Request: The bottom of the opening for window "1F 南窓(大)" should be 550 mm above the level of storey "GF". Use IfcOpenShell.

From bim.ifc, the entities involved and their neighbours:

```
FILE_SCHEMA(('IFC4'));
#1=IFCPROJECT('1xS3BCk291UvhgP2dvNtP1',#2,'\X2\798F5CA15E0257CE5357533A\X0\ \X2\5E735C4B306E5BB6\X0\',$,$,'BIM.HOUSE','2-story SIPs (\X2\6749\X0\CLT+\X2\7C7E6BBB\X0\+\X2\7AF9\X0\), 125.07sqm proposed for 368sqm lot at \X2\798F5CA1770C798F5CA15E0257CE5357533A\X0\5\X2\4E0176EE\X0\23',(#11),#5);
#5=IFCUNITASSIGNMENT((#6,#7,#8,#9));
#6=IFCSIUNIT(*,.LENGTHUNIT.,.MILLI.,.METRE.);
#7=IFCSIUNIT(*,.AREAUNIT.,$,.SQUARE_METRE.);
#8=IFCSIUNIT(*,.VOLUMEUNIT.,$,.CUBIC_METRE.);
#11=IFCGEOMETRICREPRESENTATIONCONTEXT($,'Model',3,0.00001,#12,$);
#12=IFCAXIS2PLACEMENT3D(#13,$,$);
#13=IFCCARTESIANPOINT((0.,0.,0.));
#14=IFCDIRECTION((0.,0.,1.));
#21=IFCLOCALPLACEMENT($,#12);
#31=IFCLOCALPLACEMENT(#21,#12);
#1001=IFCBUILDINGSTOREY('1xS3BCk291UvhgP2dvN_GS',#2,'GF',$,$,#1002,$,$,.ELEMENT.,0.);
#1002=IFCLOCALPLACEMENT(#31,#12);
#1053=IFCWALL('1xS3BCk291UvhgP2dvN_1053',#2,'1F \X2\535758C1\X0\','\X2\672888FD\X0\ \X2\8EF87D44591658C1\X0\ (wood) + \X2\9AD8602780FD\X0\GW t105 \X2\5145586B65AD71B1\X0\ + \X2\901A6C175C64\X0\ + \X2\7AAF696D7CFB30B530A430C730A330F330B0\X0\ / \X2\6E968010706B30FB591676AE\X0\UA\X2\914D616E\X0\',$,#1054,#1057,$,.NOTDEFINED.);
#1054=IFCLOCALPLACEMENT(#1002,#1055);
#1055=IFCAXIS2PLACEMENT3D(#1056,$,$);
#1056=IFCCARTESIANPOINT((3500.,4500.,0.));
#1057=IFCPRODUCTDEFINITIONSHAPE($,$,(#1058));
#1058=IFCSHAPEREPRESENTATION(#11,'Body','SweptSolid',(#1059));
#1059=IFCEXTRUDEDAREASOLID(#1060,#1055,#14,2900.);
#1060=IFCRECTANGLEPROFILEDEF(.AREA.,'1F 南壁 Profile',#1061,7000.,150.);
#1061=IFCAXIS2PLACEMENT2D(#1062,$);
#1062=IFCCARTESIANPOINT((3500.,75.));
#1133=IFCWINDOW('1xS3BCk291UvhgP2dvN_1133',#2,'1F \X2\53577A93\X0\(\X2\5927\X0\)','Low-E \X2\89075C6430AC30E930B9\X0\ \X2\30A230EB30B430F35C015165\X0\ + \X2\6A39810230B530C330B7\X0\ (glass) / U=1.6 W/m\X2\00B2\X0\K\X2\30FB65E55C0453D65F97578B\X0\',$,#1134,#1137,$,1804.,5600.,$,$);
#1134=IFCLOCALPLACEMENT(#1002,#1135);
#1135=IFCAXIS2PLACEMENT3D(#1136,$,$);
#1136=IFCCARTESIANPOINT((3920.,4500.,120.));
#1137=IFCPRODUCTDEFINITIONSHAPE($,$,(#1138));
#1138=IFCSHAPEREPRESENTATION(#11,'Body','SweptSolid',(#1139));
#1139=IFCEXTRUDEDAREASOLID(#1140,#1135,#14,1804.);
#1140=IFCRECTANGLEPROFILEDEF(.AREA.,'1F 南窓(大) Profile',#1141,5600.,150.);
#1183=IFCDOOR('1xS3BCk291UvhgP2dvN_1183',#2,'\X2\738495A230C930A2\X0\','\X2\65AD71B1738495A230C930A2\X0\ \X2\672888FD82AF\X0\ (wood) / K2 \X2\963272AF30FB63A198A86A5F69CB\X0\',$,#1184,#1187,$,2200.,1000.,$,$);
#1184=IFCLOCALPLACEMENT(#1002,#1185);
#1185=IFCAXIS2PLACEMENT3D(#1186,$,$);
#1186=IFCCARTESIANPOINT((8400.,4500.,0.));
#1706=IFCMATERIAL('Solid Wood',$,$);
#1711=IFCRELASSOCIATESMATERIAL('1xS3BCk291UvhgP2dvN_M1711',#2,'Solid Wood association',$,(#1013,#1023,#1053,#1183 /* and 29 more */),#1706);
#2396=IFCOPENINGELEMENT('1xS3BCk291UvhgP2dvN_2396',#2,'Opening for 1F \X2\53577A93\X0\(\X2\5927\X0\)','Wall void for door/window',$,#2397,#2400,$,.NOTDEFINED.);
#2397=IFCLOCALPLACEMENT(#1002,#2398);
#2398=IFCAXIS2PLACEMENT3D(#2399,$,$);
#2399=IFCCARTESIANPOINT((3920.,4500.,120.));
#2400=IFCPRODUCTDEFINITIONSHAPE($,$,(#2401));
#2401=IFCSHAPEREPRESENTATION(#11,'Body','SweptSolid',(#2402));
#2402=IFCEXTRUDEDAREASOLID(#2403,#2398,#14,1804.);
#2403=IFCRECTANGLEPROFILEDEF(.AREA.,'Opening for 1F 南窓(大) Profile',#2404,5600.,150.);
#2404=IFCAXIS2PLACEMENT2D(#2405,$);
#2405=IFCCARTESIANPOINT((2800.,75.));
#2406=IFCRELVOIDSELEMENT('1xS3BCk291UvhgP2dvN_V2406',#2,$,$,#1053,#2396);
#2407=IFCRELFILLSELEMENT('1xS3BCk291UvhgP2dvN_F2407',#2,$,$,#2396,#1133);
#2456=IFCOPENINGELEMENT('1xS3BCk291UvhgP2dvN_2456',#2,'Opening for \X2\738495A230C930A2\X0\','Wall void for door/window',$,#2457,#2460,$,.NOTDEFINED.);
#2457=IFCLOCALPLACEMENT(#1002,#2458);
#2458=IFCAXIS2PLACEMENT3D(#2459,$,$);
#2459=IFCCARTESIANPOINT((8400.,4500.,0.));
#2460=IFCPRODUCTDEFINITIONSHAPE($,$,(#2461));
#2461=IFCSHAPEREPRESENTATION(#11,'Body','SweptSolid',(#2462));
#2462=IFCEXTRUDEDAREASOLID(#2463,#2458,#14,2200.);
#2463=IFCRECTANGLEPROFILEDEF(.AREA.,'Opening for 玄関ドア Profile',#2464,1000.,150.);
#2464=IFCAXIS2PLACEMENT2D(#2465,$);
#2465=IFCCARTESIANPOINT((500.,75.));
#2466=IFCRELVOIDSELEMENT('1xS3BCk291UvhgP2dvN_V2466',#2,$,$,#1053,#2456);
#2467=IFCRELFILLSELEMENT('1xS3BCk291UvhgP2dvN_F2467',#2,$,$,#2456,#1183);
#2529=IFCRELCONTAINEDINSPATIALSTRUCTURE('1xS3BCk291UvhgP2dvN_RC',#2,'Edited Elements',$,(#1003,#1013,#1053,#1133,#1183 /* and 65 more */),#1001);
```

```python
import numpy as np
import ifcopenshell
import ifcopenshell.api.geometry
import ifcopenshell.geom
import ifcopenshell.util.element
import ifcopenshell.util.placement
import ifcopenshell.util.shape
import ifcopenshell.util.unit

model = ifcopenshell.open("bim.ifc")
unit_scale = ifcopenshell.util.unit.calculate_unit_scale(model)

window = model.by_guid("1xS3BCk291UvhgP2dvN_1133")
opening = window.FillsVoids[0].RelatingOpeningElement
storey = ifcopenshell.util.element.get_container(window, ifc_class="IfcBuildingStorey")
level = ifcopenshell.util.placement.get_local_placement(storey.ObjectPlacement)[2, 3]

# The opening's origin need not be at the sill, so measure its lowest point.
shape = ifcopenshell.geom.create_shape(ifcopenshell.geom.settings(), opening)
bottom = ifcopenshell.util.shape.get_shape_bottom_elevation(shape, shape.geometry) / unit_scale
dz = level + 550.0 - bottom

shift = np.array([0.0, 0.0, dz])
# The window is not placed relative to its opening, so move both.
for product in (opening, window):
    matrix = ifcopenshell.util.placement.get_local_placement(product.ObjectPlacement)
    matrix[:3, 3] += shift
    ifcopenshell.api.geometry.edit_object_placement(model, product=product, matrix=matrix, is_si=False)

print(f"moved by {dz * unit_scale:+.3f} m")

model.write("bim_updated.ifc")
```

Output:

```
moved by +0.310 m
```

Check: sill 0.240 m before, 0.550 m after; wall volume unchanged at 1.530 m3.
